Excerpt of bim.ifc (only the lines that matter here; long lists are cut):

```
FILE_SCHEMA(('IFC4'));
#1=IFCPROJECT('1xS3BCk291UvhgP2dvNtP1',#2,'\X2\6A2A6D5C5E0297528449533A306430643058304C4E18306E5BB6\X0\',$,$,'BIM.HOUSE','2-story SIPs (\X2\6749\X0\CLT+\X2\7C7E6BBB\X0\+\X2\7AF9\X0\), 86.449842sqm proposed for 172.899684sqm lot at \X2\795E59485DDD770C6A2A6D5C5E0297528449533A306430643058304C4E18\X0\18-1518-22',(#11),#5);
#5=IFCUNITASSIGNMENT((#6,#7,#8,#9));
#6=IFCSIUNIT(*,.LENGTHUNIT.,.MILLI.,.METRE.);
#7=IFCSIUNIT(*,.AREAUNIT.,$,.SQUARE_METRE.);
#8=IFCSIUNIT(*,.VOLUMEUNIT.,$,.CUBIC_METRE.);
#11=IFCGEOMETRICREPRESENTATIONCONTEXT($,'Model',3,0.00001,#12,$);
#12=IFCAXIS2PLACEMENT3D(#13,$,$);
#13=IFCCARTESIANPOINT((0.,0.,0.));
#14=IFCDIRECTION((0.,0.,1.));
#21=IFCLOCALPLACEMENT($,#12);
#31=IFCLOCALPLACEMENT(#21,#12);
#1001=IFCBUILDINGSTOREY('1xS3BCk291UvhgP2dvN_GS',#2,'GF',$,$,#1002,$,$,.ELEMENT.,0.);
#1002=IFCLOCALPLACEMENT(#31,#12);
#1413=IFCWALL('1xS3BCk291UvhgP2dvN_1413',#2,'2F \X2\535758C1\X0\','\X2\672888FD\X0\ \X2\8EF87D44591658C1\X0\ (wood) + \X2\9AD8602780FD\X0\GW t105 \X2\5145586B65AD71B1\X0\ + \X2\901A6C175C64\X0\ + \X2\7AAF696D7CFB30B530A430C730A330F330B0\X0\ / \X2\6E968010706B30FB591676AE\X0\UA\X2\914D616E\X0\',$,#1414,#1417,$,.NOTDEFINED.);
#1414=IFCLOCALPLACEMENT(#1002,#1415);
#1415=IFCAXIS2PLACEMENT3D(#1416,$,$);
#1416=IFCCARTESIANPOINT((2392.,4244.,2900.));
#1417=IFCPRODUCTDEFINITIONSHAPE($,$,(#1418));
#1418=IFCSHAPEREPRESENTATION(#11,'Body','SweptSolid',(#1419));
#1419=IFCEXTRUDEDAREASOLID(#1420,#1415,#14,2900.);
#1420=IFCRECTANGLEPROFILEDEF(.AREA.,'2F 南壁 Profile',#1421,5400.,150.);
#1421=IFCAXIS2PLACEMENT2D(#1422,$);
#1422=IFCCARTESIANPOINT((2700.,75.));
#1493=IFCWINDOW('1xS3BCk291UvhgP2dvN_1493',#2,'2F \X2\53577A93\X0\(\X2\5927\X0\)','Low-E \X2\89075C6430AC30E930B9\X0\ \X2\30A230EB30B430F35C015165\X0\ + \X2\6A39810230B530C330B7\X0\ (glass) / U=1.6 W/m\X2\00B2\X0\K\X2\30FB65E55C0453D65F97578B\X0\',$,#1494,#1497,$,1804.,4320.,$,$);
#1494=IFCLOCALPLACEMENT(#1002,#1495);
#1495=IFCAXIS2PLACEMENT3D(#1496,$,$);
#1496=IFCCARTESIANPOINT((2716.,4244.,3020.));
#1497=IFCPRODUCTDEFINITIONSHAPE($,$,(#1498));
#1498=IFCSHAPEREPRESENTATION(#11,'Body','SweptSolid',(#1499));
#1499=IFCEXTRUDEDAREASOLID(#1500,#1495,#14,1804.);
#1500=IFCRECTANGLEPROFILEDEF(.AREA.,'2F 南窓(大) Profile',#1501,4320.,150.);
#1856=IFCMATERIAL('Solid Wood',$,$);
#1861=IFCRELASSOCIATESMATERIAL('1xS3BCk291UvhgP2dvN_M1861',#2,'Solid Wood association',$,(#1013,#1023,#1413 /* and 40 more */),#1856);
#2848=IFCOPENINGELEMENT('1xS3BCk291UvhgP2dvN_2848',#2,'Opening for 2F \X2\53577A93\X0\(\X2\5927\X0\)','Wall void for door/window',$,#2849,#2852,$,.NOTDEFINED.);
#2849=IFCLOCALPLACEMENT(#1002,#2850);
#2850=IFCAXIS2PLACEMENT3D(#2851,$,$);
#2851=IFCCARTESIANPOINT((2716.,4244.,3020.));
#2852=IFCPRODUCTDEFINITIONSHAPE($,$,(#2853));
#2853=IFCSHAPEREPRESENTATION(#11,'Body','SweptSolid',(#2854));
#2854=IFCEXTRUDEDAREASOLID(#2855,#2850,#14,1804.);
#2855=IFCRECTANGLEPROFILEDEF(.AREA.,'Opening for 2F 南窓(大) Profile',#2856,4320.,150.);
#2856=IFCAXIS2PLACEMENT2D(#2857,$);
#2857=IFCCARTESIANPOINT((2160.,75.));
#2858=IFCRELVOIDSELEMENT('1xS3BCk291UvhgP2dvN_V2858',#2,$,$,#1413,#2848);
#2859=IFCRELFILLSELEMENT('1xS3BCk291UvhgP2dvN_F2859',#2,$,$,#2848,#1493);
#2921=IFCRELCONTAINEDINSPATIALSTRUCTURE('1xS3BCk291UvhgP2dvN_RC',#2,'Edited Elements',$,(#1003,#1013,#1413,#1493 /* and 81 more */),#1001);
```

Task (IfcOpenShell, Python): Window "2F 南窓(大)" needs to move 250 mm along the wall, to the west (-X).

```python
import ifcopenshell
import ifcopenshell.api.geometry
import ifcopenshell.util.placement

model = ifcopenshell.open("bim.ifc")

window = model.by_guid("1xS3BCk291UvhgP2dvN_1493")
opening = window.FillsVoids[0].RelatingOpeningElement
wall = opening.VoidsElements[0].RelatingBuildingElement

wall_matrix = ifcopenshell.util.placement.get_local_placement(wall.ObjectPlacement)
shift = wall_matrix[:3, 0] * -250.0
before = ifcopenshell.util.placement.get_local_placement(window.ObjectPlacement)[:3, 3].copy()

# The window is not placed relative to its opening, so move both.
for product in (opening, window):
    matrix = ifcopenshell.util.placement.get_local_placement(product.ObjectPlacement)
    matrix[:3, 3] += shift
    ifcopenshell.api.geometry.edit_object_placement(model, product=product, matrix=matrix, is_si=False)

after = ifcopenshell.util.placement.get_local_placement(window.ObjectPlacement)[:3, 3]
print("window moved by", (after - before).round(3) + 0.0)

model.write("bim_v2.ifc")
```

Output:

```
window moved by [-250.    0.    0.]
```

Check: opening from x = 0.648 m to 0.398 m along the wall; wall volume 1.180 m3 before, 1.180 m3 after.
